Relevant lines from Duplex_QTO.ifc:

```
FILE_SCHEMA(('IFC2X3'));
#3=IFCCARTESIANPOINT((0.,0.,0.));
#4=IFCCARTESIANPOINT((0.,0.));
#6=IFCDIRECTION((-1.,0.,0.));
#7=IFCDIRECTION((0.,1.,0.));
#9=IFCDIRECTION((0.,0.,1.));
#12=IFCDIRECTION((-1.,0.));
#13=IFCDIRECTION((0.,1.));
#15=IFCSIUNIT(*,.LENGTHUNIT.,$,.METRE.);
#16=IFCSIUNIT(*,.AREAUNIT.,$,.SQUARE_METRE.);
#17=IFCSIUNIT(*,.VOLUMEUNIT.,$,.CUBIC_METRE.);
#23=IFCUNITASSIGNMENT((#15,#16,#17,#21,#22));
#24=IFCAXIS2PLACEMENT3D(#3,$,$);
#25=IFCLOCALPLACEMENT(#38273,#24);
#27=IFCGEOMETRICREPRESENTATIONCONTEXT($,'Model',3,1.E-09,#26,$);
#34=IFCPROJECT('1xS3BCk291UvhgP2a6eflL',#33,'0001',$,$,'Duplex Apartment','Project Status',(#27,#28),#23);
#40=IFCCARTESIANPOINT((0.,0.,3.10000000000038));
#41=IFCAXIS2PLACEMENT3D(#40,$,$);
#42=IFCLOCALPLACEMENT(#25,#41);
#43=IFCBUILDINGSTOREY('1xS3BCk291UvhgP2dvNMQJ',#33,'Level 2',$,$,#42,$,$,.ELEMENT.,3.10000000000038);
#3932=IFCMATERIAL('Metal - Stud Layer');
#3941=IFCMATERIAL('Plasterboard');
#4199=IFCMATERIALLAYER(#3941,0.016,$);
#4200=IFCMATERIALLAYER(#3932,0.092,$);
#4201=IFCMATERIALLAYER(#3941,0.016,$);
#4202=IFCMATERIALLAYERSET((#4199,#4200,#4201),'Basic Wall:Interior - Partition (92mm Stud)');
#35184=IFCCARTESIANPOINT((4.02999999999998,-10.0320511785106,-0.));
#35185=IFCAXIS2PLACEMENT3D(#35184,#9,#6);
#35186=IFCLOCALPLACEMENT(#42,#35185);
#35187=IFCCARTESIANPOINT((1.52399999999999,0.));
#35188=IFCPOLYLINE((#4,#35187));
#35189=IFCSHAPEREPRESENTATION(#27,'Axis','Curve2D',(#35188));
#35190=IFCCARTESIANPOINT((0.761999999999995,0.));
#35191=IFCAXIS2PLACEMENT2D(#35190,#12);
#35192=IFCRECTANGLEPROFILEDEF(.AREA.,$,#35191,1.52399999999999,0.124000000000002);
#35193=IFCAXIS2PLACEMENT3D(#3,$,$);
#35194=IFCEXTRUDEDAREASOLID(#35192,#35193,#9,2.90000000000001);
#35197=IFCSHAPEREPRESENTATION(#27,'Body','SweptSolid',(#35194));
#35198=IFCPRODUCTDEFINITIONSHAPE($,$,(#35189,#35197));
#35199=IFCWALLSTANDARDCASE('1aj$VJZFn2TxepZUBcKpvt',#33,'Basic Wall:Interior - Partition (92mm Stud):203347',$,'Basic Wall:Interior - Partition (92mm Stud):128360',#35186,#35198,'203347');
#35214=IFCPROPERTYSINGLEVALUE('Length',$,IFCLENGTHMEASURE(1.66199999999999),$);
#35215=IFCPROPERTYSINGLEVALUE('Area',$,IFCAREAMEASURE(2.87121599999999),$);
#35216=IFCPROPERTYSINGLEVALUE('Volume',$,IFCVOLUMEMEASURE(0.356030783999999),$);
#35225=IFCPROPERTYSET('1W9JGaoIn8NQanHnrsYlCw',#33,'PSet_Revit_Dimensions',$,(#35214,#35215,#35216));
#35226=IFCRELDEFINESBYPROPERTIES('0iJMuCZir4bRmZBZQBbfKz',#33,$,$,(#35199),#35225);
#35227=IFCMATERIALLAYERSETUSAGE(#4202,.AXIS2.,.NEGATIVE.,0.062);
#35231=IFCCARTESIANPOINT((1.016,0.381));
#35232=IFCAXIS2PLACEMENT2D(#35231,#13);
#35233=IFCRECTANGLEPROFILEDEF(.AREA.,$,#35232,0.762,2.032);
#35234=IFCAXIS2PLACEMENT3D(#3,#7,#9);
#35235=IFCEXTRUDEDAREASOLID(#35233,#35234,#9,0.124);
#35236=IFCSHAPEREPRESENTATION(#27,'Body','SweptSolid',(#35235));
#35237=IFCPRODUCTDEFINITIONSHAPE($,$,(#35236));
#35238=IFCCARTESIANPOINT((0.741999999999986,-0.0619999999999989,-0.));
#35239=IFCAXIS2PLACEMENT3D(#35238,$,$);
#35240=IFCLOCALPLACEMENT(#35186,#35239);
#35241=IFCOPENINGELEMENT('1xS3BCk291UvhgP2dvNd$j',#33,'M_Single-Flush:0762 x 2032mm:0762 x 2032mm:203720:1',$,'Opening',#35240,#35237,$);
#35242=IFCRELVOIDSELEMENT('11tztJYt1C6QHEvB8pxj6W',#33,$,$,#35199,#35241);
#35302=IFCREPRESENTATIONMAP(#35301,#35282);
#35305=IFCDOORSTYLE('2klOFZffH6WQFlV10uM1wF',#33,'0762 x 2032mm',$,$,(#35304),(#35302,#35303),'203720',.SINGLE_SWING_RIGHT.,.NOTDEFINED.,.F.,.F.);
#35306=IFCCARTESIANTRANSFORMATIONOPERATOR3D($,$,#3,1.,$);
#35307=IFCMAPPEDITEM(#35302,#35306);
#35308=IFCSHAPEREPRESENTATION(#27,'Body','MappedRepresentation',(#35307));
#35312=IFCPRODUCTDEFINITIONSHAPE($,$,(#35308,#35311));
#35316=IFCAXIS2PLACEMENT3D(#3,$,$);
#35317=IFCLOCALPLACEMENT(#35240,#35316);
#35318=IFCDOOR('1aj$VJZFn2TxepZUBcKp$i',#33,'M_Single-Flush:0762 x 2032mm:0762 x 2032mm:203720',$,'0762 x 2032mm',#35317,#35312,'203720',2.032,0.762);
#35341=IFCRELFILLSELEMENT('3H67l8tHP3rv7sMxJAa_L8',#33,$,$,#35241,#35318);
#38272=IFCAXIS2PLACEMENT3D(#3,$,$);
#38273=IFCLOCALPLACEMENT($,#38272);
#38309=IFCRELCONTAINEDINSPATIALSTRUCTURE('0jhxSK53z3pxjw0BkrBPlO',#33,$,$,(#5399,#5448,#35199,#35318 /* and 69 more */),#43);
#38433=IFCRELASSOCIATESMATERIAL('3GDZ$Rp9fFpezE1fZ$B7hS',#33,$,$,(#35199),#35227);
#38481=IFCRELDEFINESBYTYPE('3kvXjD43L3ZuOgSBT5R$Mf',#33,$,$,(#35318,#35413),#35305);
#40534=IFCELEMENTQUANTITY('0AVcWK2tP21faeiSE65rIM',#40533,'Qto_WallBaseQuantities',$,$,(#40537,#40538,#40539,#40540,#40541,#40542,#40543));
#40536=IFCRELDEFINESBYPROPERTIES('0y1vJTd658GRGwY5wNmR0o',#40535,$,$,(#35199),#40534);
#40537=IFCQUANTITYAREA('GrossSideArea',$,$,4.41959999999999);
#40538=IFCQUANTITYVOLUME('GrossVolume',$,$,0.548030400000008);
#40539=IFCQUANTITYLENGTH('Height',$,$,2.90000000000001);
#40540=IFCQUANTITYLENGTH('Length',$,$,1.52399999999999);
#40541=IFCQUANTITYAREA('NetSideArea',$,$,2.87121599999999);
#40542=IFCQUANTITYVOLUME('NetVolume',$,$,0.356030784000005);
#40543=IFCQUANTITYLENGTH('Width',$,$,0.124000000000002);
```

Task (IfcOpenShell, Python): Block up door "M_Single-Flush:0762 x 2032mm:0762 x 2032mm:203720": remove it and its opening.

```python
import ifcopenshell
import ifcopenshell.api.feature
import ifcopenshell.api.pset
import ifcopenshell.api.root
import ifcopenshell.geom
import ifcopenshell.util.element
import ifcopenshell.util.shape
import ifcopenshell.util.unit

model = ifcopenshell.open("Duplex_QTO.ifc")
area_scale = ifcopenshell.util.unit.calculate_unit_scale(model, "AREAUNIT")
volume_scale = ifcopenshell.util.unit.calculate_unit_scale(model, "VOLUMEUNIT")
settings = ifcopenshell.geom.settings()


def volume(element):
    """Net volume in cubic metres, openings subtracted."""
    shape = ifcopenshell.geom.create_shape(settings, element)
    return ifcopenshell.util.shape.get_volume(shape.geometry)


door = model.by_id(35318)
opening = door.FillsVoids[0].RelatingOpeningElement
wall = opening.VoidsElements[0].RelatingBuildingElement
before = volume(wall)

ifcopenshell.api.root.remove_product(model, product=door)
ifcopenshell.api.feature.remove_feature(model, feature=opening)

after = volume(wall)
thickness = 0.124  # wall thickness in metres

# Update the wall's stored quantities.
pset = model.by_id(ifcopenshell.util.element.get_pset(wall, "PSet_Revit_Dimensions", should_inherit=False)["id"])
ifcopenshell.api.pset.edit_pset(model, pset=pset, properties={
    "Area": model.create_entity("IfcAreaMeasure", after / thickness / area_scale),
    "Volume": model.create_entity("IfcVolumeMeasure", after / volume_scale),
})
qto = model.by_id(ifcopenshell.util.element.get_pset(wall, "Qto_WallBaseQuantities", should_inherit=False)["id"])
ifcopenshell.api.pset.edit_qto(model, qto=qto, properties={
    "NetSideArea": after / thickness / area_scale,
    "NetVolume": after / volume_scale,
})

print(f"wall volume {before:.3f} -> {after:.3f} m3")

model.write("Duplex_QTO-out.ifc")
```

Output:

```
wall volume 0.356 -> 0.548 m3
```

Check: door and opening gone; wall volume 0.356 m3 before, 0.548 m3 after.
